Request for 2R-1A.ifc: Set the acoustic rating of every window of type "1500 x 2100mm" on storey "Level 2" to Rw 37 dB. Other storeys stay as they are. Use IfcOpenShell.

First a look at what the model holds.

```python
import ifcopenshell
import ifcopenshell.util.element

model = ifcopenshell.open("2R-1A.ifc")
print(model.schema)
storey = next(s for s in model.by_type("IfcBuildingStorey") if s.Name == "Level 2")
windows = [e for e in ifcopenshell.util.element.get_decomposition(storey) if e.is_a("IfcWindow")]
seen = {}
for e in windows:
    element_type = ifcopenshell.util.element.get_type(e)
    key = (element_type.Name if element_type != e and element_type else None, ifcopenshell.util.element.get_pset(e, "Pset_WindowCommon", "AcousticRating"))
    seen[key] = seen.get(key, 0) + 1
for (name, value), count in sorted(seen.items(), key=str):
    print(count, "x", name, "|", value)
```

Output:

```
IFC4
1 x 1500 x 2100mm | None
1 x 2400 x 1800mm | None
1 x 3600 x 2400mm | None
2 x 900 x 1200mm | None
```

```python
import ifcopenshell
import ifcopenshell.api.pset
import ifcopenshell.util.element

model = ifcopenshell.open("2R-1A.ifc")

storey = next(s for s in model.by_type("IfcBuildingStorey") if s.Name == "Level 2")
windows = [e for e in ifcopenshell.util.element.get_decomposition(storey) if e.is_a("IfcWindow")]

count = 0
for e in windows:
    element_type = ifcopenshell.util.element.get_type(e)
    if element_type in (None, e) or element_type.Name != "1500 x 2100mm":
        continue
    # add_pset returns the element's existing set when there is one.
    pset = ifcopenshell.api.pset.add_pset(model, product=e, name="Pset_WindowCommon")
    ifcopenshell.api.pset.edit_pset(model, pset=pset, properties={"AcousticRating": "Rw 37 dB"})
    count += 1

print(count, "windows updated")

model.write("2R-1A_updated.ifc")
```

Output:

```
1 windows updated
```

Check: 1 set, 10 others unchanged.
